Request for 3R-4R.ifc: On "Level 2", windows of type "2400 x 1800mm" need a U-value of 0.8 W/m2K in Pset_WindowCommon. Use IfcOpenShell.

First a look at what the model holds.

```python
import ifcopenshell
import ifcopenshell.util.element

model = ifcopenshell.open("3R-4R.ifc")
print(model.schema)
storey = next(s for s in model.by_type("IfcBuildingStorey") if s.Name == "Level 2")
windows = [e for e in ifcopenshell.util.element.get_decomposition(storey) if e.is_a("IfcWindow")]
seen = {}
for e in windows:
    element_type = ifcopenshell.util.element.get_type(e)
    key = (element_type.Name if element_type != e and element_type else None, ifcopenshell.util.element.get_pset(e, "Pset_WindowCommon", "ThermalTransmittance"))
    seen[key] = seen.get(key, 0) + 1
for (name, value), count in sorted(seen.items(), key=str):
    print(count, "x", name, "|", value)
```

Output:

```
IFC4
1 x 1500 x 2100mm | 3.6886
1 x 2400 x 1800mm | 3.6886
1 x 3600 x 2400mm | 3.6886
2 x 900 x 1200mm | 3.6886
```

```python
import ifcopenshell
import ifcopenshell.api.pset
import ifcopenshell.util.element

model = ifcopenshell.open("3R-4R.ifc")

storey = next(s for s in model.by_type("IfcBuildingStorey") if s.Name == "Level 2")
windows = [e for e in ifcopenshell.util.element.get_decomposition(storey) if e.is_a("IfcWindow")]

count = 0
for e in windows:
    element_type = ifcopenshell.util.element.get_type(e)
    if element_type in (None, e) or element_type.Name != "2400 x 1800mm":
        continue
    # add_pset returns the element's existing set when there is one.
    pset = ifcopenshell.api.pset.add_pset(model, product=e, name="Pset_WindowCommon")
    ifcopenshell.api.pset.edit_pset(model, pset=pset, properties={"ThermalTransmittance": 0.8})
    count += 1

print(count, "windows updated")

model.write("3R-4R-out.ifc")
```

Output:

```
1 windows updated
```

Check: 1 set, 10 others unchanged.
